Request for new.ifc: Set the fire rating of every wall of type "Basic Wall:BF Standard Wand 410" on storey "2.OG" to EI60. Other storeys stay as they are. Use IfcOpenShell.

First a look at what the model holds.

```python
import ifcopenshell
import ifcopenshell.util.element

model = ifcopenshell.open("new.ifc")
print(model.schema)
storey = next(s for s in model.by_type("IfcBuildingStorey") if s.Name == "2.OG")
walls = [e for e in ifcopenshell.util.element.get_decomposition(storey) if e.is_a("IfcWall")]
seen = {}
for e in walls:
    element_type = ifcopenshell.util.element.get_type(e)
    key = (element_type.Name if element_type != e and element_type else None, ifcopenshell.util.element.get_pset(e, "Pset_WallCommon", "FireRating"))
    seen[key] = seen.get(key, 0) + 1
for (name, value), count in sorted(seen.items(), key=str):
    print(count, "x", name, "|", value)
```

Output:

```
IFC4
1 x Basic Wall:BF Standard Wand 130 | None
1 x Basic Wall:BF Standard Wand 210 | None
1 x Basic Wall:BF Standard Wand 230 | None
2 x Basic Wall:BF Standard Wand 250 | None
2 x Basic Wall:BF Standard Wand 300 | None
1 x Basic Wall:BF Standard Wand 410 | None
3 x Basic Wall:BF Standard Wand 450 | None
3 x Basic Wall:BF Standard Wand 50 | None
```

```python
import ifcopenshell
import ifcopenshell.api.pset
import ifcopenshell.util.element

model = ifcopenshell.open("new.ifc")

storey = next(s for s in model.by_type("IfcBuildingStorey") if s.Name == "2.OG")
walls = [e for e in ifcopenshell.util.element.get_decomposition(storey) if e.is_a("IfcWall")]

count = 0
for e in walls:
    element_type = ifcopenshell.util.element.get_type(e)
    if element_type in (None, e) or element_type.Name != "Basic Wall:BF Standard Wand 410":
        continue
    # add_pset returns the element's existing set when there is one.
    pset = ifcopenshell.api.pset.add_pset(model, product=e, name="Pset_WallCommon")
    ifcopenshell.api.pset.edit_pset(model, pset=pset, properties={"FireRating": "EI60"})
    count += 1

print(count, "walls updated")

model.write("new_updated.ifc")
```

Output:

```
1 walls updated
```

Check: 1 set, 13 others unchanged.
